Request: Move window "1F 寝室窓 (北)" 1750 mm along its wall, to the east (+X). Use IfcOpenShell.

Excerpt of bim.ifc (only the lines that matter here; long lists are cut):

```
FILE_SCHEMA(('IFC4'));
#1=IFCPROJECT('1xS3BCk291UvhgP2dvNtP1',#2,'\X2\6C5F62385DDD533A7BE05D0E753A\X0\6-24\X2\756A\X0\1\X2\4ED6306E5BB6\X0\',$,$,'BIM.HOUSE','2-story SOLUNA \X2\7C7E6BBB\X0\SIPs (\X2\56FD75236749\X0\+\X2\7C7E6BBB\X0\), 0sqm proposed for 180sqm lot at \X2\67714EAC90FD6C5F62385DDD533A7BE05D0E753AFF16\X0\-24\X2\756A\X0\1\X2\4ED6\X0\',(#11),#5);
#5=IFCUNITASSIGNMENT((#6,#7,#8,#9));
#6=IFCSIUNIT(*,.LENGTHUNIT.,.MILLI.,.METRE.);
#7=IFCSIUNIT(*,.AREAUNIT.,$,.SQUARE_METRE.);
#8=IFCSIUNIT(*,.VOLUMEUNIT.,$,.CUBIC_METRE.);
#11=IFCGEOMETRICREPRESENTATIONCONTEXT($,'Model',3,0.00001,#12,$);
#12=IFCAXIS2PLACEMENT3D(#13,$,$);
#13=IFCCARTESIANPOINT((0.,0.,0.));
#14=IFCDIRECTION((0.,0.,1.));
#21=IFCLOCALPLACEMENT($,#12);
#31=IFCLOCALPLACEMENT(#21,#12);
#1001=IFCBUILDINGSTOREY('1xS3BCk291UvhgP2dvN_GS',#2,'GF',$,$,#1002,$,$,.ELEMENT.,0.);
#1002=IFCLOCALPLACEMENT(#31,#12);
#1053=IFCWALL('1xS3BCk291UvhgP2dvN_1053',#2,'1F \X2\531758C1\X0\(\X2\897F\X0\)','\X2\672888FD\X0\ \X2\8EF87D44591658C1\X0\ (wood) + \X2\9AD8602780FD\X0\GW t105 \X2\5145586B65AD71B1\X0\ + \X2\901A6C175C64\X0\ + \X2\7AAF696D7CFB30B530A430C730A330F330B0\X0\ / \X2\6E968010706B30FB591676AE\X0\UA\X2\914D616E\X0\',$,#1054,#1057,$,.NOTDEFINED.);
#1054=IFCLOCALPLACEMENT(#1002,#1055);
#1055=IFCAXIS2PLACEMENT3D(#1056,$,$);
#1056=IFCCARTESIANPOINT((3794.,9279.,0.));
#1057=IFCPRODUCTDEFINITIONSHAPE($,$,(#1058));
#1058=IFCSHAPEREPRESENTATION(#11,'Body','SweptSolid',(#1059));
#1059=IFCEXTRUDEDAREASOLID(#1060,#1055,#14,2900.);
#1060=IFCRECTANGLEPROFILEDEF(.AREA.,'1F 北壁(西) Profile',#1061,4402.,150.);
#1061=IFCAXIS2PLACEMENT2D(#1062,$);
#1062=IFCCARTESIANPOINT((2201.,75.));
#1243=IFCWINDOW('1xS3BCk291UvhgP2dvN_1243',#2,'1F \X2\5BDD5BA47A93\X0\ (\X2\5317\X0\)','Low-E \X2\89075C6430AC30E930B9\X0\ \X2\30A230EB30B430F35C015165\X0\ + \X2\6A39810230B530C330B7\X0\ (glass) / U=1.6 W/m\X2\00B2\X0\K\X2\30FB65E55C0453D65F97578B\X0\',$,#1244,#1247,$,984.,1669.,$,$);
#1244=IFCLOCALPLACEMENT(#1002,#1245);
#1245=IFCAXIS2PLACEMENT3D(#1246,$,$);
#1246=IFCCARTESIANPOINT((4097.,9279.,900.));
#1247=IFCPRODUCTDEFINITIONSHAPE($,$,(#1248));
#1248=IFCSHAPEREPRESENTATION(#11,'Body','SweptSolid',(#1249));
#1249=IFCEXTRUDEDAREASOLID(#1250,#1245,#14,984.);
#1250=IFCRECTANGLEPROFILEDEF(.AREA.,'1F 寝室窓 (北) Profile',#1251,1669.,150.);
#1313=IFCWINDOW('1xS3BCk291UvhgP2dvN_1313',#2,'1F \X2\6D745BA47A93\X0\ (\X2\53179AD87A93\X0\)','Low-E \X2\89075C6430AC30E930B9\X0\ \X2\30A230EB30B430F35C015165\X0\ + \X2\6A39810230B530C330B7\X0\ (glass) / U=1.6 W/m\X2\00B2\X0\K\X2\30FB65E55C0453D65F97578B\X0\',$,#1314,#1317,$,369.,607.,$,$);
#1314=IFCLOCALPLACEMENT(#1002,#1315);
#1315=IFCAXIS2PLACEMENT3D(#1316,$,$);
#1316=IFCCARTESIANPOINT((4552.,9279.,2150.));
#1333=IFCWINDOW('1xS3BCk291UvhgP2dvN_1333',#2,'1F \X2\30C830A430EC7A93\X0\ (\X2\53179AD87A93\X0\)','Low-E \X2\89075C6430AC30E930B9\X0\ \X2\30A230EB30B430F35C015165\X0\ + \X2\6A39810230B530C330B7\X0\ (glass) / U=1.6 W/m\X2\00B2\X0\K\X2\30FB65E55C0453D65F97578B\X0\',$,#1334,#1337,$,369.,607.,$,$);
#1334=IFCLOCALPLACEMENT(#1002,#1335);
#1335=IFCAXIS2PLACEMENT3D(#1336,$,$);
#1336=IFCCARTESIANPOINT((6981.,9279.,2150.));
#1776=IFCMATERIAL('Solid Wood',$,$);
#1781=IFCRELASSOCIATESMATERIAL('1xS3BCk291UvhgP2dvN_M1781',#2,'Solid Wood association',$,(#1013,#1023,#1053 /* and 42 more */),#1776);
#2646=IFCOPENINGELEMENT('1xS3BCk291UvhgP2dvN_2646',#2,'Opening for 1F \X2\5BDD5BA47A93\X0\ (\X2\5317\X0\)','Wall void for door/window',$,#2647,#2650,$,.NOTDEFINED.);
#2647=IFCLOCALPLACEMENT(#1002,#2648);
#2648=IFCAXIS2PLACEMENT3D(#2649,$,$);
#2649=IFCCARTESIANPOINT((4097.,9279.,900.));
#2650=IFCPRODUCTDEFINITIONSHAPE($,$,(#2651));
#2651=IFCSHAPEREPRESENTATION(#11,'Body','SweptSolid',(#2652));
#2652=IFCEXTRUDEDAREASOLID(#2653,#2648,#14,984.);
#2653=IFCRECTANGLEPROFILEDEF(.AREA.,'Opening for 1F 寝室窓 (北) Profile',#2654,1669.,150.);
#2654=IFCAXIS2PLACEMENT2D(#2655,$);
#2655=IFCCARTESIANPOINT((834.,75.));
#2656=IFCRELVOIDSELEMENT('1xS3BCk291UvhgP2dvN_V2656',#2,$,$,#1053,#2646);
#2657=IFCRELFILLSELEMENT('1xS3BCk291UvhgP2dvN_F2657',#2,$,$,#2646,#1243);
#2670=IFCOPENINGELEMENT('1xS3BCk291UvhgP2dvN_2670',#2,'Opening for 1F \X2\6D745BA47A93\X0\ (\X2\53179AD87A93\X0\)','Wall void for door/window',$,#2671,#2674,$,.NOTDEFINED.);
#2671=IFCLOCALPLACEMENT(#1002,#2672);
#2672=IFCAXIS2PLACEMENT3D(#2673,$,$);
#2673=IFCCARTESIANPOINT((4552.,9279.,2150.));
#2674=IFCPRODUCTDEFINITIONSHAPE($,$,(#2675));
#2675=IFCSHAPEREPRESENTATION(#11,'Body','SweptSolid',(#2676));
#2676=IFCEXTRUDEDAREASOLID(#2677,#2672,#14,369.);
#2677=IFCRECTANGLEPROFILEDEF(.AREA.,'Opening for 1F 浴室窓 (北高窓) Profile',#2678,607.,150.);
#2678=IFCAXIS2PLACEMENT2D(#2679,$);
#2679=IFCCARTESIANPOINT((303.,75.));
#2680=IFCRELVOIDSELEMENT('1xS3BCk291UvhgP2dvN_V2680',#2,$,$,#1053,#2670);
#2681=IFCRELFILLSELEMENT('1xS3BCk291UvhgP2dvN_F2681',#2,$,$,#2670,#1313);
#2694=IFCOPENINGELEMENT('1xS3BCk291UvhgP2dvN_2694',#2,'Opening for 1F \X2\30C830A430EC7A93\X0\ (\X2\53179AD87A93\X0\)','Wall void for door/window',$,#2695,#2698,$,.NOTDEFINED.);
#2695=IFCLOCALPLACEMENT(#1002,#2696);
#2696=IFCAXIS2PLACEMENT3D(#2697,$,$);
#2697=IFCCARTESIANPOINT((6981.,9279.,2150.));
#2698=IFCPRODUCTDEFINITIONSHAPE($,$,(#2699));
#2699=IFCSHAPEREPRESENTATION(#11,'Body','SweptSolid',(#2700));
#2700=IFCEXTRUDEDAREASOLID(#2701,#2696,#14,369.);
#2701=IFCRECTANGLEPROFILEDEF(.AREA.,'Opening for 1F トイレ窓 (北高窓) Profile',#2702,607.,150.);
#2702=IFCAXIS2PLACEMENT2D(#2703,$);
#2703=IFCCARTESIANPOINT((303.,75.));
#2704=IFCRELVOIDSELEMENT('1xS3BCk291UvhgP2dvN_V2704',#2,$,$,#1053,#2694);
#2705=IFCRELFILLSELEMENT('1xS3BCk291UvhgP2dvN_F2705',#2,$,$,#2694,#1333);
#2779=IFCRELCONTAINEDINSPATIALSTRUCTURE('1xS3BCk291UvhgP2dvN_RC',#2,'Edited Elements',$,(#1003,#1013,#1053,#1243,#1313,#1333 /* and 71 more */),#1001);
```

```python
import ifcopenshell
import ifcopenshell.api.geometry
import ifcopenshell.util.placement
import ifcopenshell.util.unit

model = ifcopenshell.open("bim.ifc")
unit_scale = ifcopenshell.util.unit.calculate_unit_scale(model)

window = model.by_id(1243)
opening = window.FillsVoids[0].RelatingOpeningElement
wall = opening.VoidsElements[0].RelatingBuildingElement

wall_matrix = ifcopenshell.util.placement.get_local_placement(wall.ObjectPlacement)
shift = wall_matrix[:3, 0] * 1.75 / unit_scale
before = ifcopenshell.util.placement.get_local_placement(window.ObjectPlacement)[:3, 3].copy()

# The window is not placed relative to its opening, so move both.
for product in (opening, window):
    matrix = ifcopenshell.util.placement.get_local_placement(product.ObjectPlacement)
    matrix[:3, 3] += shift
    ifcopenshell.api.geometry.edit_object_placement(model, product=product, matrix=matrix, is_si=False)

after = ifcopenshell.util.placement.get_local_placement(window.ObjectPlacement)[:3, 3]
print("window moved by", (after - before).round(3) + 0.0)

model.write("bim_updated.ifc")
```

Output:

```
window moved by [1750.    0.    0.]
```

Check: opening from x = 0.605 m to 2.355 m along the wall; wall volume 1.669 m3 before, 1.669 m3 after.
